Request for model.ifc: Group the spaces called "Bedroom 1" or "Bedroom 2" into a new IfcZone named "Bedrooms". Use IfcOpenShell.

First a look at what the model holds.

```python
import ifcopenshell

model = ifcopenshell.open("model.ifc")
print(model.schema)
seen = {}
for space in model.by_type("IfcSpace"):
    seen[space.LongName] = seen.get(space.LongName, 0) + 1
for name, count in sorted(seen.items(), key=str):
    print(count, "x", name)
print("zones:", [z.Name for z in model.by_type("IfcZone")][:20])
```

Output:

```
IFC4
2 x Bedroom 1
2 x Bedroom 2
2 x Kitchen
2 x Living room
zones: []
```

```python
import ifcopenshell
import ifcopenshell.api.group
import ifcopenshell.api.root

model = ifcopenshell.open("model.ifc")

names = {"Bedroom 1", "Bedroom 2"}
spaces = [s for s in model.by_type("IfcSpace") if s.LongName in names]

zone = ifcopenshell.api.root.create_entity(model, ifc_class="IfcZone", name="Bedrooms")
ifcopenshell.api.group.assign_group(model, products=spaces, group=zone)
print(len(spaces), "spaces in", zone.Name)

model.write("model_updated.ifc")
```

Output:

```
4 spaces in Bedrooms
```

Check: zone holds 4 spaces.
